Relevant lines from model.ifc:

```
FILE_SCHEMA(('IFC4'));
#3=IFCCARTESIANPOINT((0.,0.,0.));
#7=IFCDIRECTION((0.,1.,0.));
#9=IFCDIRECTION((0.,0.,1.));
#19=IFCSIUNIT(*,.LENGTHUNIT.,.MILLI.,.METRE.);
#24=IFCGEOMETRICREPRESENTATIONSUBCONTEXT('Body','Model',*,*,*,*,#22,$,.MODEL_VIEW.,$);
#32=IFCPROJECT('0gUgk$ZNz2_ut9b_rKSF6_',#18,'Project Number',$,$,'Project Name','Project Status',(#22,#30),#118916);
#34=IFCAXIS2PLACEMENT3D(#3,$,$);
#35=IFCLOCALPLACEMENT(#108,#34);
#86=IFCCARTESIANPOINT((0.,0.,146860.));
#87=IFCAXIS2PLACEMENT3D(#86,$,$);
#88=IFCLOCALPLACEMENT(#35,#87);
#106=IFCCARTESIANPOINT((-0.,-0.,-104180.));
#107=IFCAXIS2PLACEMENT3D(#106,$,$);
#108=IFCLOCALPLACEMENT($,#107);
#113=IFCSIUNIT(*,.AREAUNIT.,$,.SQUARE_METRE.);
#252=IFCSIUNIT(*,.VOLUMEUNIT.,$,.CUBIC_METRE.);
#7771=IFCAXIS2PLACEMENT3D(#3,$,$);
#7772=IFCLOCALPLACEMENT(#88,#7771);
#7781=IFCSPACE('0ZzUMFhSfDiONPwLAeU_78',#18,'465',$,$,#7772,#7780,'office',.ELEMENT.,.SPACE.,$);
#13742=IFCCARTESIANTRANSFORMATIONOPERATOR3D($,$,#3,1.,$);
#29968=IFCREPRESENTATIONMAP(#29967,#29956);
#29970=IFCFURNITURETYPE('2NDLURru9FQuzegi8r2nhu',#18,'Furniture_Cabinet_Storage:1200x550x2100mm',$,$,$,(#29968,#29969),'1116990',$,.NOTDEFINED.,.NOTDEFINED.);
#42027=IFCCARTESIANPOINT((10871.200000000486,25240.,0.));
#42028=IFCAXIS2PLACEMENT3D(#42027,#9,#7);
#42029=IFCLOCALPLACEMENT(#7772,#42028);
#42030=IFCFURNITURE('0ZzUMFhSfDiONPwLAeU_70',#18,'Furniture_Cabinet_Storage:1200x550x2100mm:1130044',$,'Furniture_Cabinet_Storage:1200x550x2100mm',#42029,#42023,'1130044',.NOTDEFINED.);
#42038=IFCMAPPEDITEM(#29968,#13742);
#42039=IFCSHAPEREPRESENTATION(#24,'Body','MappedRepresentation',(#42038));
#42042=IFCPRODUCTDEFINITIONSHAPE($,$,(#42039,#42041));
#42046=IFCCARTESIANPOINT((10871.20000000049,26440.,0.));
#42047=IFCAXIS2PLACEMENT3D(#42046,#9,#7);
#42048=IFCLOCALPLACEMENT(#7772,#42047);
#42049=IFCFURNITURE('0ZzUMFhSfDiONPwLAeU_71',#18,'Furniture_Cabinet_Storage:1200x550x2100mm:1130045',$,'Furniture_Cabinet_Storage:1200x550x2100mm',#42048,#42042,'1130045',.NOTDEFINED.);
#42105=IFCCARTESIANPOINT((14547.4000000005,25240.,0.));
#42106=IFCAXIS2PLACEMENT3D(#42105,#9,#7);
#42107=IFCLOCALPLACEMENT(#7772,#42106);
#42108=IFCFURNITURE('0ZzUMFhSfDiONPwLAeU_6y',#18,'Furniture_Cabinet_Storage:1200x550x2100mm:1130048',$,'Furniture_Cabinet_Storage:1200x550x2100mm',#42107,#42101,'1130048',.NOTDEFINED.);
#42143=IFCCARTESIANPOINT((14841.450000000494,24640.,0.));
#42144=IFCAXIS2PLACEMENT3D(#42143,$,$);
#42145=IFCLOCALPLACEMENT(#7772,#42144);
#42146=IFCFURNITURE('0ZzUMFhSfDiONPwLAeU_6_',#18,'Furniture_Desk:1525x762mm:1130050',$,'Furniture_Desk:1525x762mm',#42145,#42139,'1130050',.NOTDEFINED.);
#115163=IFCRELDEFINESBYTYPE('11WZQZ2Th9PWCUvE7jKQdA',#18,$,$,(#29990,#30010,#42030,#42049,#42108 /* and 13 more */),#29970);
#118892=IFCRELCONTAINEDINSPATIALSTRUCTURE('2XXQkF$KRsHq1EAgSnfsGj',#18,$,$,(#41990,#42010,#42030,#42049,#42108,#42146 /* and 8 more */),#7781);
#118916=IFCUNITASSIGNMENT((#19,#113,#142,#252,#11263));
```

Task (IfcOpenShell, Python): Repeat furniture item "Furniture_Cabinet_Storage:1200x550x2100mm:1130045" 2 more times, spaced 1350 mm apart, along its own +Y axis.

```python
import ifcopenshell
import ifcopenshell.api.geometry
import ifcopenshell.api.root
import ifcopenshell.util.element
import ifcopenshell.util.placement

model = ifcopenshell.open("model.ifc")


def reuse_history(source, copy):
    """copy_class also copies each property set's owner history, people and application; keep the originals."""
    for rel in copy.IsDefinedBy:
        if rel.is_a("IfcRelDefinesByProperties") and (history := rel.RelatingPropertyDefinition.OwnerHistory):
            rel.RelatingPropertyDefinition.OwnerHistory = source.OwnerHistory
            ifcopenshell.util.element.remove_deep2(model, history)


source = model.by_guid("0ZzUMFhSfDiONPwLAeU_71")
base = ifcopenshell.util.placement.get_local_placement(source.ObjectPlacement)
step = base[:3, 1] * 1350.0

for i in range(1, 3):
    copy = ifcopenshell.api.root.copy_class(model, product=source)
    copy.Representation = ifcopenshell.util.element.copy_deep(
        model, source.Representation, exclude=["IfcGeometricRepresentationContext", "IfcRepresentationMap"]
    )
    copy.Name = "Furniture_Cabinet_Storage:1200x550x2100mm"
    copy.Tag = None
    reuse_history(source, copy)
    matrix = base.copy()
    matrix[:3, 3] += i * step
    print("added at", matrix[:3, 3].round(3) + 0.0)
    ifcopenshell.api.geometry.edit_object_placement(model, product=copy, matrix=matrix, is_si=False)

model.write("model_v2.ifc")
```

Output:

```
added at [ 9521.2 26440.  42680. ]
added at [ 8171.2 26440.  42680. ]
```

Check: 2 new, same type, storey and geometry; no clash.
